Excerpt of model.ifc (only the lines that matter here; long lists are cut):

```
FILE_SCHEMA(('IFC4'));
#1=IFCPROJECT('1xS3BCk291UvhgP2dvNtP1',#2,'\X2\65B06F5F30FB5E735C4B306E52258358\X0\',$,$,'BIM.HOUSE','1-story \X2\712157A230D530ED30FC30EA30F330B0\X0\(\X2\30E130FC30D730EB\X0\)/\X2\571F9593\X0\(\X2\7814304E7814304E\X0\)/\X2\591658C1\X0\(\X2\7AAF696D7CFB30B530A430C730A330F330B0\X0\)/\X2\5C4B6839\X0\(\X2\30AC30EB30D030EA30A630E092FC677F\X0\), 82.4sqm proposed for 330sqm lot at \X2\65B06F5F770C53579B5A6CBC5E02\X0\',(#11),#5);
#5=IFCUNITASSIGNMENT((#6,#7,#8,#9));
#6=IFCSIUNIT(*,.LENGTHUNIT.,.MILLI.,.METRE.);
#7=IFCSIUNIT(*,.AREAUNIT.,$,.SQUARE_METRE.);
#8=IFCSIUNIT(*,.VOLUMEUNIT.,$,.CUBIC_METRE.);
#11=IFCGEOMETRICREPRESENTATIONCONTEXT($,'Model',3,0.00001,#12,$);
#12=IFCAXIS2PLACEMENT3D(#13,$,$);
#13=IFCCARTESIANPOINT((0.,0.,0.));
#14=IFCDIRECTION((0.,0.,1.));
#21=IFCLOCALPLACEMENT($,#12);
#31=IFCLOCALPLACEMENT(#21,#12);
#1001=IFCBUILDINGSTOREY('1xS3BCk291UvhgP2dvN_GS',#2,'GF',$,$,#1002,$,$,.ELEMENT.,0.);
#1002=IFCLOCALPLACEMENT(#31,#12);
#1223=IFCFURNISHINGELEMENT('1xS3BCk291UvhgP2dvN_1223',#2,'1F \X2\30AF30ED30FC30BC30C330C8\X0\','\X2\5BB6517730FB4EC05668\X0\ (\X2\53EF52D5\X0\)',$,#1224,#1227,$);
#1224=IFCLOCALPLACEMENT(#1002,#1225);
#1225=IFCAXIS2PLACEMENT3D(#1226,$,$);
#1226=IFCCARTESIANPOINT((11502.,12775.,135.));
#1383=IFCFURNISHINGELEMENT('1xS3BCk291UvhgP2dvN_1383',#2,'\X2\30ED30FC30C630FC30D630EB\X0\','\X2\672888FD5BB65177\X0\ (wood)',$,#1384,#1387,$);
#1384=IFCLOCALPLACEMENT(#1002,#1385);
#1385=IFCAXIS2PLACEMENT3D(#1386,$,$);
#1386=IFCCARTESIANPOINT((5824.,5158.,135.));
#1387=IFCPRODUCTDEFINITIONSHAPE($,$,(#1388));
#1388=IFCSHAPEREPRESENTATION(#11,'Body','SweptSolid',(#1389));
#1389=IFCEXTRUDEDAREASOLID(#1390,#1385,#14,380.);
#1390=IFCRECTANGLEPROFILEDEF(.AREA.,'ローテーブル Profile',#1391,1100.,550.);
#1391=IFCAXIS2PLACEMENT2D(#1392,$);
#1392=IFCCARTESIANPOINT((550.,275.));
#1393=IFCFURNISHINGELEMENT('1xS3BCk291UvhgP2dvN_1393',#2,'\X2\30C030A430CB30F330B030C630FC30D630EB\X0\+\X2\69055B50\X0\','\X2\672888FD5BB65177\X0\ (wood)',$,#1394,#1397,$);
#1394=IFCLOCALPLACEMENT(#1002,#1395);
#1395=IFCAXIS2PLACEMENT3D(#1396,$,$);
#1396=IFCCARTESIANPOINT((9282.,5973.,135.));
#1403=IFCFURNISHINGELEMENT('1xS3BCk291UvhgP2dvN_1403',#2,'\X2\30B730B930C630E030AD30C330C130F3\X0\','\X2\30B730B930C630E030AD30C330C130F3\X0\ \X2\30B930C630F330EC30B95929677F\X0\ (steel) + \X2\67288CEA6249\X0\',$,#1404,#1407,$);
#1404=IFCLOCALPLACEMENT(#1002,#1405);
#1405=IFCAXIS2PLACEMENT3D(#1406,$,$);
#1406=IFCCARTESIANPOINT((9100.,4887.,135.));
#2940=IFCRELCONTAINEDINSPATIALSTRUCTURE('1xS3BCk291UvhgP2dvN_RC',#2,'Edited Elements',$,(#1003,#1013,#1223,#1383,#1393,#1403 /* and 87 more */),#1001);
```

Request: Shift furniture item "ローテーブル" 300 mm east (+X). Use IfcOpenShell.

```python
import ifcopenshell
import ifcopenshell.api.geometry
import ifcopenshell.util.placement
import ifcopenshell.util.unit

model = ifcopenshell.open("model.ifc")
unit_scale = ifcopenshell.util.unit.calculate_unit_scale(model)

item = model.by_id(1383)
matrix = ifcopenshell.util.placement.get_local_placement(item.ObjectPlacement)
matrix[0, 3] += 0.3 / unit_scale
ifcopenshell.api.geometry.edit_object_placement(model, product=item, matrix=matrix, is_si=False)

print(ifcopenshell.util.placement.get_local_placement(item.ObjectPlacement).round(3) + 0.0)

model.write("model_rev.ifc")
```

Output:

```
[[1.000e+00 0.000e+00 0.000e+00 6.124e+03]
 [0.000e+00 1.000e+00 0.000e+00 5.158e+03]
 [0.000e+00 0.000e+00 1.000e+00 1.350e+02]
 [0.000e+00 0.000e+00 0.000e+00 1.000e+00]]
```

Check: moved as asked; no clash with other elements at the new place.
